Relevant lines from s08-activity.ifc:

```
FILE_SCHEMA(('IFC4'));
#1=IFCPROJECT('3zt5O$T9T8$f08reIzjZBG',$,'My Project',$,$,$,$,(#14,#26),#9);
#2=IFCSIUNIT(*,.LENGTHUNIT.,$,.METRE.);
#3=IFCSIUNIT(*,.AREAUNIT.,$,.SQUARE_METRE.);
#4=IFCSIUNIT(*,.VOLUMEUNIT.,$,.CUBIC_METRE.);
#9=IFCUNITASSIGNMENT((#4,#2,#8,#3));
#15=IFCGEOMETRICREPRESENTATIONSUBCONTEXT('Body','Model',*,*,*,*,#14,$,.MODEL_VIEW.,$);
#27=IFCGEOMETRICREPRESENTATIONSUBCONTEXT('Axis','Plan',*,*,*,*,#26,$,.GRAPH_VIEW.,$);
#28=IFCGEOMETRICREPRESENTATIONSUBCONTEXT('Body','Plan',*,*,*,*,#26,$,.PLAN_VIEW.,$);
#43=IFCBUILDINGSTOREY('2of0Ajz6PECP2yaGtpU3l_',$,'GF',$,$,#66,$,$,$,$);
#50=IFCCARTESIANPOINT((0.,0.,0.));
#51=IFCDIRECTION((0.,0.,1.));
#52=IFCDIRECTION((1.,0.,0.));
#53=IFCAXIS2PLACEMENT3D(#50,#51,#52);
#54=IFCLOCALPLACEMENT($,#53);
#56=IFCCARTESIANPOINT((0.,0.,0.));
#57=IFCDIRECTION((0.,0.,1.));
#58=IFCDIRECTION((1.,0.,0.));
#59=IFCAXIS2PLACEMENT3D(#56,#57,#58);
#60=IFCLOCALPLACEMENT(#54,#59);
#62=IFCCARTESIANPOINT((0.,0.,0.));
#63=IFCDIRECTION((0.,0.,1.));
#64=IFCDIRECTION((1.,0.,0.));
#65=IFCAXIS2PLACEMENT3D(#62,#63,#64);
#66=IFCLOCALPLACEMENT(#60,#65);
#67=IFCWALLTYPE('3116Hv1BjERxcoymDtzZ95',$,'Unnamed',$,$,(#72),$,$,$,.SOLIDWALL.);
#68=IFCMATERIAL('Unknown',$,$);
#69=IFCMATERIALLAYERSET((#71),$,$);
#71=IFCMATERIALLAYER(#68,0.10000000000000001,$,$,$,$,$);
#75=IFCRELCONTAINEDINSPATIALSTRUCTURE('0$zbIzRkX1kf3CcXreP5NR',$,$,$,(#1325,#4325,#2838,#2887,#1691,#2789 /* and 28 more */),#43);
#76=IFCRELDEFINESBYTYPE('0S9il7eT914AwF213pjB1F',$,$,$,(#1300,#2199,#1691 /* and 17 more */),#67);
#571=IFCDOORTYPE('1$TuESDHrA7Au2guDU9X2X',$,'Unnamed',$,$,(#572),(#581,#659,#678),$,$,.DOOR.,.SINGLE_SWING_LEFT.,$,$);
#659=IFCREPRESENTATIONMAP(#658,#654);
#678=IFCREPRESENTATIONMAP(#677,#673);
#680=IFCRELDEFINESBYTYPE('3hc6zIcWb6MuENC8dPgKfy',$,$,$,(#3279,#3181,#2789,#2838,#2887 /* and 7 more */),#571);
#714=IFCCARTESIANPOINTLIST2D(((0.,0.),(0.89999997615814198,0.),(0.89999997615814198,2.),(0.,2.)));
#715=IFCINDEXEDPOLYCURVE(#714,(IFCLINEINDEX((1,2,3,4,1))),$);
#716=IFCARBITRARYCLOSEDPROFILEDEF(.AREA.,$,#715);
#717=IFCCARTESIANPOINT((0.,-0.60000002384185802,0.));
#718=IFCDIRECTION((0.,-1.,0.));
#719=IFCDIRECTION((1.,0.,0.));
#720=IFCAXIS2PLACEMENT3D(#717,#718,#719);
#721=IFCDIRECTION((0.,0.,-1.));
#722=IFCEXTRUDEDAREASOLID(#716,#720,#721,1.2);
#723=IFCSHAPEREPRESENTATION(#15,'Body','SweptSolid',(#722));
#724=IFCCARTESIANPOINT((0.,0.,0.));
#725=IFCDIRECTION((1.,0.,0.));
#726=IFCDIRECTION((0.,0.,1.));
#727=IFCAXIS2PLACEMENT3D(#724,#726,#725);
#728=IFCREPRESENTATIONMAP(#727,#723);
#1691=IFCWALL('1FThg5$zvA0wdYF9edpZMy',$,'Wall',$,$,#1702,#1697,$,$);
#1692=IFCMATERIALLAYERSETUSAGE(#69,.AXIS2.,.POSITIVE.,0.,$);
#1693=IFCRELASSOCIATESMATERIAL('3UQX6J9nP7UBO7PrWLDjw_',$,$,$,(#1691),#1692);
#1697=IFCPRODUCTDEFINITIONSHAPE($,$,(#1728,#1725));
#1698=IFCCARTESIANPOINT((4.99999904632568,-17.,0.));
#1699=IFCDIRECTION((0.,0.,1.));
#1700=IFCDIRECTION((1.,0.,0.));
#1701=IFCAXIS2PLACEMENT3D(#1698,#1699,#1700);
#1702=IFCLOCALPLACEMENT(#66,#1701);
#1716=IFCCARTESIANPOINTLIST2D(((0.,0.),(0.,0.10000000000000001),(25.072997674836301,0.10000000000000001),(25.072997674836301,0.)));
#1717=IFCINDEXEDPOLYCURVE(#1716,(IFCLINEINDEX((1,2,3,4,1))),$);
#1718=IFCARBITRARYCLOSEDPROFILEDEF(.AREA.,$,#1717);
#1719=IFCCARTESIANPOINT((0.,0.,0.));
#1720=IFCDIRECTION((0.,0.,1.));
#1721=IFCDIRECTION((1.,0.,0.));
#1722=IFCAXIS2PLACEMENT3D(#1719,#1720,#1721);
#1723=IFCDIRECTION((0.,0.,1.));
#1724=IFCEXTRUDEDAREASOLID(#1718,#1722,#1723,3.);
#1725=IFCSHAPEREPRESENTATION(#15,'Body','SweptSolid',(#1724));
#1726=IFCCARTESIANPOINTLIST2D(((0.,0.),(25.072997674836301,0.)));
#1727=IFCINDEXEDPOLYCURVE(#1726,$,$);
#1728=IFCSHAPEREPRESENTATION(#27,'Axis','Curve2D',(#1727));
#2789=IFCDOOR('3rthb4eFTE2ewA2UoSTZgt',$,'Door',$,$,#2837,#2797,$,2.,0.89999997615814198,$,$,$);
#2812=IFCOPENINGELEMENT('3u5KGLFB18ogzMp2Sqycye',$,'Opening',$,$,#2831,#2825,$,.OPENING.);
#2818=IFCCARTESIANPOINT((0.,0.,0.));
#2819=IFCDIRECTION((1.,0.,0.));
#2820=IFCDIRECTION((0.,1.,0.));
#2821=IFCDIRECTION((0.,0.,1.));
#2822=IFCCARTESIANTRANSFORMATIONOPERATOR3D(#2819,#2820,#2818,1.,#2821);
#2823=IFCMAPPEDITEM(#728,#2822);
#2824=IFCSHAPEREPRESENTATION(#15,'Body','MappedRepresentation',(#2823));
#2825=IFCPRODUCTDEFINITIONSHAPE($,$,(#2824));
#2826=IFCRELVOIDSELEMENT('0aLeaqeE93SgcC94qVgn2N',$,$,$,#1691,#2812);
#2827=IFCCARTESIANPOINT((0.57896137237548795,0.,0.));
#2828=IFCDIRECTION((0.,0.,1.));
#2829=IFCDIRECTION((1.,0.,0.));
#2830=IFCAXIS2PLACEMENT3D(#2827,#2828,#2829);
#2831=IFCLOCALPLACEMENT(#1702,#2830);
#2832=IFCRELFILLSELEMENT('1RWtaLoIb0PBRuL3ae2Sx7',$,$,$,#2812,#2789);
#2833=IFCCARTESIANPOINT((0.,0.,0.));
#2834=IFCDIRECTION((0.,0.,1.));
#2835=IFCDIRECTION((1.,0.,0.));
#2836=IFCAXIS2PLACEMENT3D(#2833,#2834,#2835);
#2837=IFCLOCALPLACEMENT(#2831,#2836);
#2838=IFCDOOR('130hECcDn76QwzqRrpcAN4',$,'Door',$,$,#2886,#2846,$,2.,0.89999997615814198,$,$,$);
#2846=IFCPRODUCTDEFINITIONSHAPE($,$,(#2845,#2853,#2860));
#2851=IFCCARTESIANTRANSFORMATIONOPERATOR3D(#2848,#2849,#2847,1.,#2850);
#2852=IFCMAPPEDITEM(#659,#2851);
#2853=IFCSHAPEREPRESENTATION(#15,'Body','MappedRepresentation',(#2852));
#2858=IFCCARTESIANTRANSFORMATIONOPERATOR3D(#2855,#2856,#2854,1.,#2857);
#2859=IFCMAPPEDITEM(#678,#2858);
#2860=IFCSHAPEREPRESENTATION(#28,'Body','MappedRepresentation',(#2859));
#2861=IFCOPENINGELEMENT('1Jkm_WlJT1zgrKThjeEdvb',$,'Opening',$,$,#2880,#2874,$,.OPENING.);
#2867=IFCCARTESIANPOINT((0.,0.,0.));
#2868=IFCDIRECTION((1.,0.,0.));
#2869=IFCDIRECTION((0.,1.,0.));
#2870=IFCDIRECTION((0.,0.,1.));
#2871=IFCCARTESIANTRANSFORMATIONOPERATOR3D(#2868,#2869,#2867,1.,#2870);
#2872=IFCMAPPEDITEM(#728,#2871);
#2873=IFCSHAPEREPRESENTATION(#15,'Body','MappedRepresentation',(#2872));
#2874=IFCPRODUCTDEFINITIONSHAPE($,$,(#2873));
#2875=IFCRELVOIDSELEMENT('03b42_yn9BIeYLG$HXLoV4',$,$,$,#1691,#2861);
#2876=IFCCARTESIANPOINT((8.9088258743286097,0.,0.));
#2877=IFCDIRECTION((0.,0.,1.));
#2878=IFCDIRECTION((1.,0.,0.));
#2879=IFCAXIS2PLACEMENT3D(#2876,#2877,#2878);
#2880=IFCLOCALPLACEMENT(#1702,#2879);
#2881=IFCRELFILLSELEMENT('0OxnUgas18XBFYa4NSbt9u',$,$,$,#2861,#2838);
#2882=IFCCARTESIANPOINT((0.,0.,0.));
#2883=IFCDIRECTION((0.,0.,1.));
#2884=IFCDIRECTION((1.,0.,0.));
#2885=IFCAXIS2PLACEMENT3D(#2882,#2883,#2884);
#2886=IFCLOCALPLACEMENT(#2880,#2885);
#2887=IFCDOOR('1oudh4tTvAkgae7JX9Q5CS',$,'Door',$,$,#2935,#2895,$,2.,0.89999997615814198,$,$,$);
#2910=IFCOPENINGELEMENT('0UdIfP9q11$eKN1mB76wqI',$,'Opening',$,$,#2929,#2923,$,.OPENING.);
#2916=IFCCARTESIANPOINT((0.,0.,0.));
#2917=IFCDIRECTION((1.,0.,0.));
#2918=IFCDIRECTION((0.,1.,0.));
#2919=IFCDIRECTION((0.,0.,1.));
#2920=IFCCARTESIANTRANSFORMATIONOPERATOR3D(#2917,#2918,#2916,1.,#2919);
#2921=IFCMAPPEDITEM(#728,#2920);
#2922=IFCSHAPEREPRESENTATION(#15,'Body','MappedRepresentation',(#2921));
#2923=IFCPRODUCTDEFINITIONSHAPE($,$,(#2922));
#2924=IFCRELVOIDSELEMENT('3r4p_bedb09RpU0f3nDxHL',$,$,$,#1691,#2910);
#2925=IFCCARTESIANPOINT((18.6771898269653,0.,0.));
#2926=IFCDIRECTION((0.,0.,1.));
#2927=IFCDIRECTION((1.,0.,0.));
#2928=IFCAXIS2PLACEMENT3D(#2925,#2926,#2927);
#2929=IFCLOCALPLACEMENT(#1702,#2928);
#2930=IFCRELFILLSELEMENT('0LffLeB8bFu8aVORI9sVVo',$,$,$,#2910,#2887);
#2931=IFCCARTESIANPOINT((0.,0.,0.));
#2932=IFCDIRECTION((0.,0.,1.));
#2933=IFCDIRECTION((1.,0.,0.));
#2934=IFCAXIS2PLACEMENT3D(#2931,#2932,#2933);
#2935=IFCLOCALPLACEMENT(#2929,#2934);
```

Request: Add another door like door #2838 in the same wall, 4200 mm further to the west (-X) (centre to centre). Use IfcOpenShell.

```python
import ifcopenshell
import ifcopenshell.api.feature
import ifcopenshell.api.geometry
import ifcopenshell.api.root
import ifcopenshell.geom
import ifcopenshell.util.element
import ifcopenshell.util.placement
import ifcopenshell.util.shape

model = ifcopenshell.open("s08-activity.ifc")
settings = ifcopenshell.geom.settings()


def volume(element):
    """Net volume in cubic metres, openings subtracted."""
    shape = ifcopenshell.geom.create_shape(settings, element)
    return ifcopenshell.util.shape.get_volume(shape.geometry)


door = model.by_guid("130hECcDn76QwzqRrpcAN4")
opening = door.FillsVoids[0].RelatingOpeningElement
wall = opening.VoidsElements[0].RelatingBuildingElement
before = volume(wall)
shift = ifcopenshell.util.placement.get_local_placement(wall.ObjectPlacement)[:3, 0] * -4.2

# copy_class copies the void relationship, type, container and properties, but no geometry.
new_opening = ifcopenshell.api.root.copy_class(model, product=opening)
new_opening.Representation = ifcopenshell.util.element.copy_deep(
    model, opening.Representation, exclude=["IfcGeometricRepresentationContext", "IfcRepresentationMap"]
)
new_door = ifcopenshell.api.root.copy_class(model, product=door)
new_door.Representation = ifcopenshell.util.element.copy_deep(
    model, door.Representation, exclude=["IfcGeometricRepresentationContext", "IfcRepresentationMap"]
)
ifcopenshell.api.feature.add_filling(model, opening=new_opening, element=new_door)

for old, new in ((opening, new_opening), (door, new_door)):
    matrix = ifcopenshell.util.placement.get_local_placement(old.ObjectPlacement)
    matrix[:3, 3] += shift
    ifcopenshell.api.geometry.edit_object_placement(model, product=new, matrix=matrix, is_si=False)

after = volume(wall)

print(f"wall volume {before:.3f} -> {after:.3f} m3")

model.write("s08-activity_updated.ifc")
```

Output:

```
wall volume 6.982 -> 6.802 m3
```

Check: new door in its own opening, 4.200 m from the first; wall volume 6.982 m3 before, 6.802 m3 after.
